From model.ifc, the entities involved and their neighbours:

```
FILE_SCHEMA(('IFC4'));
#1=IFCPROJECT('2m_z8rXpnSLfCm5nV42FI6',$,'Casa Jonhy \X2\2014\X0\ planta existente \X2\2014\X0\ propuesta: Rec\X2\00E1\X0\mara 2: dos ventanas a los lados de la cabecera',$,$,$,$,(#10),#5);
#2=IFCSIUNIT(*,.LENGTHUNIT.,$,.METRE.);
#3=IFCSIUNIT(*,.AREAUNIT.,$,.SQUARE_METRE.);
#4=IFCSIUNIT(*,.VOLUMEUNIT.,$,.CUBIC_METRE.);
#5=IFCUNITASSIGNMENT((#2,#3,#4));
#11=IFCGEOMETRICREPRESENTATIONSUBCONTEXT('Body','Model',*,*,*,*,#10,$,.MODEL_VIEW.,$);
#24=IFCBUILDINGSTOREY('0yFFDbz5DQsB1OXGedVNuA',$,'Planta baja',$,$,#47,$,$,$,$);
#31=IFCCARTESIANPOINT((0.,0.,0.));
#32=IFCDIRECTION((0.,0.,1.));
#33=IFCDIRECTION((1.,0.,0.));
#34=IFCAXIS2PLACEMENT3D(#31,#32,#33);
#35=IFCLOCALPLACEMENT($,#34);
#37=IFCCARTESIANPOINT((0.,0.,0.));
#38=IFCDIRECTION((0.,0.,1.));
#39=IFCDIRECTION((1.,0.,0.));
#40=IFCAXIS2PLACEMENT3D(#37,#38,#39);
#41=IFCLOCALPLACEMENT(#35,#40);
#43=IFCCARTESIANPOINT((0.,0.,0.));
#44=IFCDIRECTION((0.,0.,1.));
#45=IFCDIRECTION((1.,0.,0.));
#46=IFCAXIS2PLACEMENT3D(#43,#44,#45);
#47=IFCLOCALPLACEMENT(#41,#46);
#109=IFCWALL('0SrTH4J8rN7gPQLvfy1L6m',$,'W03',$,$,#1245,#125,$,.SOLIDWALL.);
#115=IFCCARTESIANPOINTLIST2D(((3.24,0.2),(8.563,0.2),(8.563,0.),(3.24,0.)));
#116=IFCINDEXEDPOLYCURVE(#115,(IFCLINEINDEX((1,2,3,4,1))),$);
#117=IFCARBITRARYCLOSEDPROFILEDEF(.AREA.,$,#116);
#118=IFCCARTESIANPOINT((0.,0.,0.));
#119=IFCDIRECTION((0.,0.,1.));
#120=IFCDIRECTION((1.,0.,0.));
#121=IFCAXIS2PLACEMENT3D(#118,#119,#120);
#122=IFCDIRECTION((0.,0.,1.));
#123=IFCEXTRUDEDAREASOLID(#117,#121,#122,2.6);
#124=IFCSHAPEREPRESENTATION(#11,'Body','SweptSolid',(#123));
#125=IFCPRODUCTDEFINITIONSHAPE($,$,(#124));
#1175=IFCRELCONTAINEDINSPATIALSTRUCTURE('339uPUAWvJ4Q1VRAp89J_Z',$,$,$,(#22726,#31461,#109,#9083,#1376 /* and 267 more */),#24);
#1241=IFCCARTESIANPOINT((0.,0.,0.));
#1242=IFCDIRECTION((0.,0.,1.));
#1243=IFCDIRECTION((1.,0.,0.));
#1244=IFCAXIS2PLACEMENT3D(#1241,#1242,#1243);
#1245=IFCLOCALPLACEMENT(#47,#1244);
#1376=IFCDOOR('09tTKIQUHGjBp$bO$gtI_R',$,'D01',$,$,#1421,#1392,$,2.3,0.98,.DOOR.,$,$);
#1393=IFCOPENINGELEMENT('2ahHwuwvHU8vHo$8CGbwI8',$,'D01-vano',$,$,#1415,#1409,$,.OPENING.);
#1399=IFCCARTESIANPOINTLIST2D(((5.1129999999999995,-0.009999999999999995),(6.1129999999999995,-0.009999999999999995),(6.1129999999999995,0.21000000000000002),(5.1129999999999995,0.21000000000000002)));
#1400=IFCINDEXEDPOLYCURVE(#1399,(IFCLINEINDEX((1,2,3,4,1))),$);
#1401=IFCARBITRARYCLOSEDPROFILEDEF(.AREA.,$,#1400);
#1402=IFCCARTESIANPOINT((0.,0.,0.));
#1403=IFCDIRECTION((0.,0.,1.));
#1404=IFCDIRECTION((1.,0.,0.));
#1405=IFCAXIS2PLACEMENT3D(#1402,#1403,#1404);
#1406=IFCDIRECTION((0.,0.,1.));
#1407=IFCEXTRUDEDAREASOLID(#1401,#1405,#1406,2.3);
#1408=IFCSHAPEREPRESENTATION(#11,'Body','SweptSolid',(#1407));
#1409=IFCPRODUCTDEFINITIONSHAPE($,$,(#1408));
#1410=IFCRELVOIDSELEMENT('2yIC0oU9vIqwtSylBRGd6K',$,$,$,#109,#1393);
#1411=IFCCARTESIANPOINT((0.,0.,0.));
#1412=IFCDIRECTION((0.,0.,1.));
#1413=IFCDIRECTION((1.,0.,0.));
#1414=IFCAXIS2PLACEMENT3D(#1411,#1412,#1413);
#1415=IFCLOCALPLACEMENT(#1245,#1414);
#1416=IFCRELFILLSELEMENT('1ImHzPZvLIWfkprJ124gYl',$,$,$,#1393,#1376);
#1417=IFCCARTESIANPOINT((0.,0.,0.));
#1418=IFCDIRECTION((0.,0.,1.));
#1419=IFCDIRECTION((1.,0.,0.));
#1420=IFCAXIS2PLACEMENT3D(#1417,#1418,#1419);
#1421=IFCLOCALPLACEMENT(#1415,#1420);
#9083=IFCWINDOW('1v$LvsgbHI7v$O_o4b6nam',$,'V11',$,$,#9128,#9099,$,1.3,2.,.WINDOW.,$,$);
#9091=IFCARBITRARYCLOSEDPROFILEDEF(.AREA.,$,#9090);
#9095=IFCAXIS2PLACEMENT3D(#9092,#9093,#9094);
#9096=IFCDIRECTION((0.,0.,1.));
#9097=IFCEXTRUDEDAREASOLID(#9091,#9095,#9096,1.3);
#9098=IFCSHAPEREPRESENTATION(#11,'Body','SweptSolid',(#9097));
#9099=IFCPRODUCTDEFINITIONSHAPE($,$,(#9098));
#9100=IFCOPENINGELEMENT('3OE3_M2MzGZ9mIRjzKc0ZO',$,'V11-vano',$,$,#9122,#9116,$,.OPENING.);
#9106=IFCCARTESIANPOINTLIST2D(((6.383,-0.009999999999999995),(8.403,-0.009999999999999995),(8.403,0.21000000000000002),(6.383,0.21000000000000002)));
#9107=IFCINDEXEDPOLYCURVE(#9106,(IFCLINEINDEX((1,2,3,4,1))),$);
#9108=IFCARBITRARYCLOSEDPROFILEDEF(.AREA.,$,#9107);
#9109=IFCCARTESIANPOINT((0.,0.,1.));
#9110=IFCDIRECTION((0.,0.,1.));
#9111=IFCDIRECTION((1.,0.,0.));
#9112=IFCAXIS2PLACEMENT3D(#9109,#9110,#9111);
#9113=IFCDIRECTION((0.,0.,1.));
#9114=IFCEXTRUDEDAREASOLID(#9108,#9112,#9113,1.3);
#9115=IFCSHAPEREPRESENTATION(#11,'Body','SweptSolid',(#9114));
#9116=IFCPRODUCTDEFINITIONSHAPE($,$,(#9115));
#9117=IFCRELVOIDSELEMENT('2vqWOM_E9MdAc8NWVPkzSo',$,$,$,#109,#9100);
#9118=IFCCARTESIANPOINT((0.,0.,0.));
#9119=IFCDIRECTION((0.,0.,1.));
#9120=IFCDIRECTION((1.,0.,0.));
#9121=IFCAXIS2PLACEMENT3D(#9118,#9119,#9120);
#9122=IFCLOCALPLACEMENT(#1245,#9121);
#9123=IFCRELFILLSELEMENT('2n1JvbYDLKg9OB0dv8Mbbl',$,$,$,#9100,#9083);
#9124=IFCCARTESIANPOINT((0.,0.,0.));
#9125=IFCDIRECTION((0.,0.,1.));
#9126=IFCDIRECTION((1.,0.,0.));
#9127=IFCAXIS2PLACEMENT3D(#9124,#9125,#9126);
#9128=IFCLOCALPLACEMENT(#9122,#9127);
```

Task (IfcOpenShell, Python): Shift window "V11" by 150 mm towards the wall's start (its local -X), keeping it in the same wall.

```python
import ifcopenshell
import ifcopenshell.api.geometry
import ifcopenshell.util.placement
import ifcopenshell.util.unit

model = ifcopenshell.open("model.ifc")
unit_scale = ifcopenshell.util.unit.calculate_unit_scale(model)

window = model.by_id(9083)
opening = window.FillsVoids[0].RelatingOpeningElement
wall = opening.VoidsElements[0].RelatingBuildingElement

wall_matrix = ifcopenshell.util.placement.get_local_placement(wall.ObjectPlacement)
shift = wall_matrix[:3, 0] * -0.15 / unit_scale
before = ifcopenshell.util.placement.get_local_placement(window.ObjectPlacement)[:3, 3].copy()

# The window is placed relative to its opening, so it follows when the opening moves.
matrix = ifcopenshell.util.placement.get_local_placement(opening.ObjectPlacement)
matrix[:3, 3] += shift
ifcopenshell.api.geometry.edit_object_placement(
    model, product=opening, matrix=matrix, is_si=False, should_transform_children=True
)

after = ifcopenshell.util.placement.get_local_placement(window.ObjectPlacement)[:3, 3]
print("window moved by", (after - before).round(3) + 0.0)

model.write("model_edited.ifc")
```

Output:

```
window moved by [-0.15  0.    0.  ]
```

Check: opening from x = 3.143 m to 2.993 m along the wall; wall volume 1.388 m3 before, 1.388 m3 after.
